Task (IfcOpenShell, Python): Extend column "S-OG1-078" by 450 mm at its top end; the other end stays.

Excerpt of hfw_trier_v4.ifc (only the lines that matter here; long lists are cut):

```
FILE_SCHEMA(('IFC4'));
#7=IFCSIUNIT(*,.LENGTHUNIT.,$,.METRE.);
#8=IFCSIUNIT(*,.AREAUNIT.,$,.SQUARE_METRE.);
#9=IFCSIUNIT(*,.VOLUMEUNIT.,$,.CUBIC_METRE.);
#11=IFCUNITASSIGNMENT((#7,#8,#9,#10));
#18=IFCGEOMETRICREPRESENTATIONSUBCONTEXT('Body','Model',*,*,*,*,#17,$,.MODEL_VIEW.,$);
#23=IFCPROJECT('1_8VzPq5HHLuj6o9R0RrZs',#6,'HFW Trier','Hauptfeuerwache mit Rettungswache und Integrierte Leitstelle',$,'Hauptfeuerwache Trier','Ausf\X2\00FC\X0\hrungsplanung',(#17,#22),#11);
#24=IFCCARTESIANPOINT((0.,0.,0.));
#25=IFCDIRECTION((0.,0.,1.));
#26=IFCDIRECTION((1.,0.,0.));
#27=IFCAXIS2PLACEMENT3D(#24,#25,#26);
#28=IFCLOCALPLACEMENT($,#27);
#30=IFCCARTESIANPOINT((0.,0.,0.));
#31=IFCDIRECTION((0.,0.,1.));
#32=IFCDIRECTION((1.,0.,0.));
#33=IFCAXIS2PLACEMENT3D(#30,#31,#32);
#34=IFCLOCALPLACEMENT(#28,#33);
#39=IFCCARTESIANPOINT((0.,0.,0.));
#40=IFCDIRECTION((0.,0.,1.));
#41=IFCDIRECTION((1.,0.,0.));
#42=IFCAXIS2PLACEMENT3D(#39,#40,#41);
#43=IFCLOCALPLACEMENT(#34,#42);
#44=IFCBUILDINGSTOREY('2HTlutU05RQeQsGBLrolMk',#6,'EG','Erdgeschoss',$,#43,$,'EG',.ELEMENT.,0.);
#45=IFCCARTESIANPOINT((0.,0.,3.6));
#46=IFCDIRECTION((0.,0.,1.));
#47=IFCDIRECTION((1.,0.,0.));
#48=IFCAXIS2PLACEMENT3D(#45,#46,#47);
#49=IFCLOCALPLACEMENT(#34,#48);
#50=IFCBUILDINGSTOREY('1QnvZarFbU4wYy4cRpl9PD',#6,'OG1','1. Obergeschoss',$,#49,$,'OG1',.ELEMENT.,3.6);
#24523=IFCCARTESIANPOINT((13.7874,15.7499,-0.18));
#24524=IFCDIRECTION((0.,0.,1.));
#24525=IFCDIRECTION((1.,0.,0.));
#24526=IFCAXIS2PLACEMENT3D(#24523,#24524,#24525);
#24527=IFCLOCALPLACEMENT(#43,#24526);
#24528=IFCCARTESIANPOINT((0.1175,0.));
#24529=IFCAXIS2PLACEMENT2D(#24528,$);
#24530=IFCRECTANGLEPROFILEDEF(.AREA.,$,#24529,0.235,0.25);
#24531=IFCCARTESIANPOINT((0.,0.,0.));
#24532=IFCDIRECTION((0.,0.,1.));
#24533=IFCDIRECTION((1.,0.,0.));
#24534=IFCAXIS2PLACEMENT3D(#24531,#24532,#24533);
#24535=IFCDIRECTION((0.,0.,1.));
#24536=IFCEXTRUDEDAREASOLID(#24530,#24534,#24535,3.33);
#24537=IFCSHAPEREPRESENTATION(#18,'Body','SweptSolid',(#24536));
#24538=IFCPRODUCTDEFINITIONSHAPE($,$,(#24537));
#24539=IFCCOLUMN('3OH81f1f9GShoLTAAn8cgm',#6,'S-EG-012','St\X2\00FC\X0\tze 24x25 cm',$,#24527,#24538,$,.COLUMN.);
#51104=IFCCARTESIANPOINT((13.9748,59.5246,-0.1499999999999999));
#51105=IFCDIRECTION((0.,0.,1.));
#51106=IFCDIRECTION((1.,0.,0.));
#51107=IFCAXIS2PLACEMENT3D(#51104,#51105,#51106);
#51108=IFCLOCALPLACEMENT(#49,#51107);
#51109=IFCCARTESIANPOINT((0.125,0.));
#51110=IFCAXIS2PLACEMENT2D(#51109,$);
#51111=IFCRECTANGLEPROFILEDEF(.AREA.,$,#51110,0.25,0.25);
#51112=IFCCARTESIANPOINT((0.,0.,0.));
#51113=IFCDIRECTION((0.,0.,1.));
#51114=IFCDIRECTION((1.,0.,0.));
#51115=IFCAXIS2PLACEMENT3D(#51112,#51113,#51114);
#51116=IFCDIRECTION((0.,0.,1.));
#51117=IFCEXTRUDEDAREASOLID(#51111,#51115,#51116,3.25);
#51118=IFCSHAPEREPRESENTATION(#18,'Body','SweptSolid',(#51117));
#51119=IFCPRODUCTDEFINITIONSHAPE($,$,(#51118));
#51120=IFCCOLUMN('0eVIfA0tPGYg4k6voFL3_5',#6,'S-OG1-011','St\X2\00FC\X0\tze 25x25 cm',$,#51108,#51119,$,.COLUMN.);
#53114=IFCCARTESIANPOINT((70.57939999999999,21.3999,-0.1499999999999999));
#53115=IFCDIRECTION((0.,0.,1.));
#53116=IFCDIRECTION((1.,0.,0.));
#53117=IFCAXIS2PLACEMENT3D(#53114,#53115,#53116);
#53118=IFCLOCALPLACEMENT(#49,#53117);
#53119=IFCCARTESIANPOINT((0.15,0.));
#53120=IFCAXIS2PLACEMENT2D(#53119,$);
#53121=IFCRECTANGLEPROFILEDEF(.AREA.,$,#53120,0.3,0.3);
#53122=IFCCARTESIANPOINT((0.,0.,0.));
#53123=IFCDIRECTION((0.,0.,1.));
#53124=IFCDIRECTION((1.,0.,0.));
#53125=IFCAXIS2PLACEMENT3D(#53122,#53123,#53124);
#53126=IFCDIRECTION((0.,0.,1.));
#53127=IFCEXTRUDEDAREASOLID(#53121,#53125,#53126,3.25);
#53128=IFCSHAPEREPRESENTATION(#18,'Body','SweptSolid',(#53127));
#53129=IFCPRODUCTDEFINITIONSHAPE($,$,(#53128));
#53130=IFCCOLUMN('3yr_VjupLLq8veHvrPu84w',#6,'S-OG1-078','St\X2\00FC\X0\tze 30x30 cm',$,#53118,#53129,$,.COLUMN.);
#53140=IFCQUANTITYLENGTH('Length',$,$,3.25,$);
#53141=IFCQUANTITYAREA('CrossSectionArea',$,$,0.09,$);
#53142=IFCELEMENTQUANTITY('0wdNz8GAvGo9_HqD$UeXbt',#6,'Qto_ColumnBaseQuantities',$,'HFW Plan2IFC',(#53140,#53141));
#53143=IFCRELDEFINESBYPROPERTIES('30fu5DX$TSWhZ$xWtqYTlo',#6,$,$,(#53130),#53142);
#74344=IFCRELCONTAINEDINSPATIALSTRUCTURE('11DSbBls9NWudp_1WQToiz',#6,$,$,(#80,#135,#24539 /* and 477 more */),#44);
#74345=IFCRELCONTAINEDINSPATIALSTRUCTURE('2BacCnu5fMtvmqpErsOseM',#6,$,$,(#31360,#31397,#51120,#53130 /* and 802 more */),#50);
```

```python
import ifcopenshell
import ifcopenshell.api.pset
import ifcopenshell.util.element
import ifcopenshell.util.representation

model = ifcopenshell.open("hfw_trier_v4.ifc")

member = model.by_guid("3yr_VjupLLq8veHvrPu84w")
change = 0.45

# The extrusion runs towards the end named, so only its depth changes.
body = ifcopenshell.util.representation.get_representation(member, "Model", "Body")
solid = body.Items[0]
old_length = solid.Depth
solid.Depth += change

# Update the stored length and volume.
qto = model.by_id(ifcopenshell.util.element.get_pset(member, "Qto_ColumnBaseQuantities", should_inherit=False)["id"])
ifcopenshell.api.pset.edit_qto(model, qto=qto, properties={"Length": solid.Depth})

print(f"length {old_length:g} -> {solid.Depth:g}")

model.write("hfw_trier_v4_rev.ifc")
```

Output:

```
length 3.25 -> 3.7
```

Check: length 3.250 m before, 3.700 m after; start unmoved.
